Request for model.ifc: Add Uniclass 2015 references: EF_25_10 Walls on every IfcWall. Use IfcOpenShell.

First a look at what the model holds.

```python
import ifcopenshell

model = ifcopenshell.open("model.ifc")
print(model.schema)
print("classifications:", [c.Name for c in model.by_type("IfcClassification")])
for ifc_class in ("IfcDoor", "IfcRoof", "IfcStair", "IfcWall", "IfcWindow"):
    print(ifc_class, len(model.by_type(ifc_class)))
```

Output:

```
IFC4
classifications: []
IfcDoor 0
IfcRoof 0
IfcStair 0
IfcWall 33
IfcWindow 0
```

```python
import ifcopenshell
import ifcopenshell.api.classification

model = ifcopenshell.open("model.ifc")

system = ifcopenshell.api.classification.add_classification(model, classification="Uniclass 2015")

codes = {
    "IfcWall": ("EF_25_10", "Walls"),
}
for ifc_class, (code, name) in codes.items():
    products = model.by_type(ifc_class)
    ifcopenshell.api.classification.add_reference(
        model, products=products, classification=system, identification=code, name=name
    )
    print(code, len(products))

model.write("model-out.ifc")
```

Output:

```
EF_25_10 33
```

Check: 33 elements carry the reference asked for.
